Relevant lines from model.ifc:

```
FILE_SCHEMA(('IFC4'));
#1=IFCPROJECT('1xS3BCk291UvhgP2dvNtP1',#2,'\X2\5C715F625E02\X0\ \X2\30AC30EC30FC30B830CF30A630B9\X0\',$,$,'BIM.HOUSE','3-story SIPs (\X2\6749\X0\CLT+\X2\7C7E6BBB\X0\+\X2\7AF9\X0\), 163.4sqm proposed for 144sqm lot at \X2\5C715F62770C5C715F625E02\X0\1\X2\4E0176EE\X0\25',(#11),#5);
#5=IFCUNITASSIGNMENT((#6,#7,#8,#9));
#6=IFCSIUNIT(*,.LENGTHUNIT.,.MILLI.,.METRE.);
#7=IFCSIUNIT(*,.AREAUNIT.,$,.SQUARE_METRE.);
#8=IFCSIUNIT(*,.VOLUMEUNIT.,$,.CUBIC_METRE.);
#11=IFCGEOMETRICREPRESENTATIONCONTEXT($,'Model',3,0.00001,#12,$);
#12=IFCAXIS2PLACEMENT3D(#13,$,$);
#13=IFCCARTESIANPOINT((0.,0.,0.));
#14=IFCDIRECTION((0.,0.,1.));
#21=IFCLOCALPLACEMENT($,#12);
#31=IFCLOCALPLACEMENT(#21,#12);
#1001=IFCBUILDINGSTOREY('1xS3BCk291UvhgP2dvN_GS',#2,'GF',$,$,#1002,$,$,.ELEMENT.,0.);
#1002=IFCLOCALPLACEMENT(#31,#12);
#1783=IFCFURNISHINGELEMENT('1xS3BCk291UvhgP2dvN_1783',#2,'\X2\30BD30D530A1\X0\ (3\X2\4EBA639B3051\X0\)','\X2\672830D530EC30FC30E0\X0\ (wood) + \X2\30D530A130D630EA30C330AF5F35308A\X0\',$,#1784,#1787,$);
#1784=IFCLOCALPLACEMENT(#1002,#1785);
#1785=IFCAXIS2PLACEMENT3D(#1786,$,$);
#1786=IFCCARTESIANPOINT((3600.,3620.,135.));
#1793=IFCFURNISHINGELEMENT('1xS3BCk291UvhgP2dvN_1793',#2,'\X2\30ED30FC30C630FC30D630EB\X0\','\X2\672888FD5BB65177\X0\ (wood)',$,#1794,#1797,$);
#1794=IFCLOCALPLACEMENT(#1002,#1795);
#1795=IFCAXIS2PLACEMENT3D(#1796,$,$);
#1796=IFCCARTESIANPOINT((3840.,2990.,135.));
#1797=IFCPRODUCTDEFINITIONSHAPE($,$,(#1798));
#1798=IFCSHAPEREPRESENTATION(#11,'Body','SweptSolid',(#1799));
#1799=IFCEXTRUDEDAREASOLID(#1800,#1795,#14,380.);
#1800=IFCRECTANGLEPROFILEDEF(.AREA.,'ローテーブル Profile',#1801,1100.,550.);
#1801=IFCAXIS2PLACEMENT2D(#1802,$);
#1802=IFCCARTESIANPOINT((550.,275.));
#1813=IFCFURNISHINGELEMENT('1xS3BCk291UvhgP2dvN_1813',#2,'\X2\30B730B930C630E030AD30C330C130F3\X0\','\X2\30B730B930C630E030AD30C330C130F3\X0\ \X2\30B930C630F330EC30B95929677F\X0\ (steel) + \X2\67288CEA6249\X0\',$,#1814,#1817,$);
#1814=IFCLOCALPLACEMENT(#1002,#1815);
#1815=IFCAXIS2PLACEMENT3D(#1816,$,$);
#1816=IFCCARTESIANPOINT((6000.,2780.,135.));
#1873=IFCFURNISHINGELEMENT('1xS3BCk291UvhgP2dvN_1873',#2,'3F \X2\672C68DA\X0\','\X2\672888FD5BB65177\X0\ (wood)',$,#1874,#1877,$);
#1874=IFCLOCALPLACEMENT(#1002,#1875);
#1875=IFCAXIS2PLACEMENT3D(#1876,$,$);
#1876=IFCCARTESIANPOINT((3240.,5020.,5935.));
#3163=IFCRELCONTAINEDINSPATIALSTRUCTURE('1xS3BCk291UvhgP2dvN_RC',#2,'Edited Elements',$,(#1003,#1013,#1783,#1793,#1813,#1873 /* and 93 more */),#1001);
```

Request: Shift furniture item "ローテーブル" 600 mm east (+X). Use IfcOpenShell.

```python
import ifcopenshell
import ifcopenshell.api.geometry
import ifcopenshell.util.placement
import ifcopenshell.util.unit

model = ifcopenshell.open("model.ifc")
unit_scale = ifcopenshell.util.unit.calculate_unit_scale(model)

item = model.by_guid("1xS3BCk291UvhgP2dvN_1793")
matrix = ifcopenshell.util.placement.get_local_placement(item.ObjectPlacement)
matrix[0, 3] += 0.6 / unit_scale
ifcopenshell.api.geometry.edit_object_placement(model, product=item, matrix=matrix, is_si=False)

print(ifcopenshell.util.placement.get_local_placement(item.ObjectPlacement).round(3) + 0.0)

model.write("model_rev.ifc")
```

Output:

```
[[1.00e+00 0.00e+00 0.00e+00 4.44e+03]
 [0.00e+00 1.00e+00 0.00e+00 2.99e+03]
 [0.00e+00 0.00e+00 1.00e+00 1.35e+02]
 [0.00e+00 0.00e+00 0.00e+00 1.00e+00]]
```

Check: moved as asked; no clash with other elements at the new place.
